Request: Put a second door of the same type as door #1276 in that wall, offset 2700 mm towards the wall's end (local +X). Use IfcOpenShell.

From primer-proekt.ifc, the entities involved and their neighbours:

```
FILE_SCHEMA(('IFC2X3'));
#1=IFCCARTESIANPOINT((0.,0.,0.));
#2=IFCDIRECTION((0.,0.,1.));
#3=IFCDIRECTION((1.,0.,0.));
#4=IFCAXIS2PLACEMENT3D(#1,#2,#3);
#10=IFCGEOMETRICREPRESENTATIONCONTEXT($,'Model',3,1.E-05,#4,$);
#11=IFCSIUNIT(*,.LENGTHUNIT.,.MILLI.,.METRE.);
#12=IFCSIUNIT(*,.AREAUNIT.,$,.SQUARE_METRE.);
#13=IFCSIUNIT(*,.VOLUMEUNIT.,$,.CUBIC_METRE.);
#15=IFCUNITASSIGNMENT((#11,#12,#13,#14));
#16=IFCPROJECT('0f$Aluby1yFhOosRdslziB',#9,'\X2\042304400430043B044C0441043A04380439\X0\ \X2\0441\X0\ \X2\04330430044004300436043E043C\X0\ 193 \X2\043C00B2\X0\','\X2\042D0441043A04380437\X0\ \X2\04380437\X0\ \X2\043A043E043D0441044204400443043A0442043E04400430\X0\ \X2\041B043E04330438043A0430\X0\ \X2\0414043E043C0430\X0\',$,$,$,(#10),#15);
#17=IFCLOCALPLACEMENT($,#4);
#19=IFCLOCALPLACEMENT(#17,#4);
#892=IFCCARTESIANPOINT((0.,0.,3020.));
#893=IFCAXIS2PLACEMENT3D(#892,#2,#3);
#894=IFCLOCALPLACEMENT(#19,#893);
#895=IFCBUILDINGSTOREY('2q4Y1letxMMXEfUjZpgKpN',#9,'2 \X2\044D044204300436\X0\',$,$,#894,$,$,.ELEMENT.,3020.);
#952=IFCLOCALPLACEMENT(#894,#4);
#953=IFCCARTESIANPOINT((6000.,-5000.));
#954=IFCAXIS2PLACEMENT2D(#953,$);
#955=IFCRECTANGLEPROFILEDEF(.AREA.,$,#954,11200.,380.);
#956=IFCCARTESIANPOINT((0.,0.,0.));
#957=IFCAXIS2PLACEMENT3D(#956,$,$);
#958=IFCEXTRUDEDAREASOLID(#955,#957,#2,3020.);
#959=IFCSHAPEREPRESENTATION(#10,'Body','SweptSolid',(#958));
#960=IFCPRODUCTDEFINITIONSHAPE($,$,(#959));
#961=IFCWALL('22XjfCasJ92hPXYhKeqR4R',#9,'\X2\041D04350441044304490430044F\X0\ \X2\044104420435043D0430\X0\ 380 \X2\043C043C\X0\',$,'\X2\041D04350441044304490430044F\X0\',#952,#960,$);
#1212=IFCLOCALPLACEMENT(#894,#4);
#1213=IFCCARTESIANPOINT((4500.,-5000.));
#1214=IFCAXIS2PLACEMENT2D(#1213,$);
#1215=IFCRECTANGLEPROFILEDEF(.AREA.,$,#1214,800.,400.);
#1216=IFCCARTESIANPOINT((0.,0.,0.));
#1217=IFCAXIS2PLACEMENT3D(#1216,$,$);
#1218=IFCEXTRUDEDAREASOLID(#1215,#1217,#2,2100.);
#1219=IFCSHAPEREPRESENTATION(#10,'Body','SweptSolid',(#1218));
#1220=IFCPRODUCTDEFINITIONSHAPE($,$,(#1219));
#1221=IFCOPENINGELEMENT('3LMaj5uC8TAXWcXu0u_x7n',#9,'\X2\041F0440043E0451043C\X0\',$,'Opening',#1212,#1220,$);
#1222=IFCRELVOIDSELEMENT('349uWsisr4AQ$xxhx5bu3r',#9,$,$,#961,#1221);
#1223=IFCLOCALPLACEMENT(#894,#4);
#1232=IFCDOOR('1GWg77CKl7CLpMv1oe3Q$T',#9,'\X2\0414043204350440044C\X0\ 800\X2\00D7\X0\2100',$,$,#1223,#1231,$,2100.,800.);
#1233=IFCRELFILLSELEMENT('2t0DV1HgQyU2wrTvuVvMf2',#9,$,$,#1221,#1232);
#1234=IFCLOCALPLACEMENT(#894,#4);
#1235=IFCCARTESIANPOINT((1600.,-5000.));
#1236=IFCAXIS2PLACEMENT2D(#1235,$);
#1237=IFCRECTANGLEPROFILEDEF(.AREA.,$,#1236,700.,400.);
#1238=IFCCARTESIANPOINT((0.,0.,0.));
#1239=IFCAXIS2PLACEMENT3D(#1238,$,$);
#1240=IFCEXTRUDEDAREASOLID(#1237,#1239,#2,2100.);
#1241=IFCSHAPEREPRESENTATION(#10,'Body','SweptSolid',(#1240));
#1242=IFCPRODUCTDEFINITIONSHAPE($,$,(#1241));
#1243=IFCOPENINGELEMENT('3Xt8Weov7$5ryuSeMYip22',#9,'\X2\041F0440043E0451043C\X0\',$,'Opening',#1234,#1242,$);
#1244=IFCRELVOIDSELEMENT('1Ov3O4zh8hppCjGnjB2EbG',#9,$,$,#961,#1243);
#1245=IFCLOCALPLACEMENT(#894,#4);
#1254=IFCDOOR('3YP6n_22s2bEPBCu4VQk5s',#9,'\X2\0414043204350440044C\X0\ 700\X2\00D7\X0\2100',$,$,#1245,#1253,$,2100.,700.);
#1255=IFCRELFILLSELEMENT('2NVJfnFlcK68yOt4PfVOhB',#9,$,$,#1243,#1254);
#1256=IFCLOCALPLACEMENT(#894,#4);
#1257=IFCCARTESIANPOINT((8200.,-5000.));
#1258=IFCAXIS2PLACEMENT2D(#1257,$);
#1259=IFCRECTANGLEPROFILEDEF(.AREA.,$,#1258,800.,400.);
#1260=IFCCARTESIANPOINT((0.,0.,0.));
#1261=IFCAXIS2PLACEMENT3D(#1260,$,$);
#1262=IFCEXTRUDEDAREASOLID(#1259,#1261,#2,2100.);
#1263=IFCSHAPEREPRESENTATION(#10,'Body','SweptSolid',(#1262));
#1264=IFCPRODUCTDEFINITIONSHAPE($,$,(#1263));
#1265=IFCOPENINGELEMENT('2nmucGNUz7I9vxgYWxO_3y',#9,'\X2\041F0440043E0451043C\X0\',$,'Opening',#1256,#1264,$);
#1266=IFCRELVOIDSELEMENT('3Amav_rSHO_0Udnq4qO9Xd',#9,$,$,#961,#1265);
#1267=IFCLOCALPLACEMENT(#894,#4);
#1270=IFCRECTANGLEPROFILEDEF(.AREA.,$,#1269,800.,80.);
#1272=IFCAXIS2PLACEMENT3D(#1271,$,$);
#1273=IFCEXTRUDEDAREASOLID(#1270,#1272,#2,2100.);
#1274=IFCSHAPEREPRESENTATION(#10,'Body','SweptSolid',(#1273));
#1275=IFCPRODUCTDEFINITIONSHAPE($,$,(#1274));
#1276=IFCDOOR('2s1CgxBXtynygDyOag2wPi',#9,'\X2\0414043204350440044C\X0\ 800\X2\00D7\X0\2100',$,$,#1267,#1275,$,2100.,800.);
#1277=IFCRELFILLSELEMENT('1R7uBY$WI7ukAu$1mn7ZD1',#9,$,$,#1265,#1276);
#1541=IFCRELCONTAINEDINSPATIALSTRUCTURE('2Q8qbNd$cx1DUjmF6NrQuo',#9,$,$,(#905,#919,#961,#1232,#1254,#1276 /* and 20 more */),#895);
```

```python
import ifcopenshell
import ifcopenshell.api.feature
import ifcopenshell.api.geometry
import ifcopenshell.api.root
import ifcopenshell.geom
import ifcopenshell.util.element
import ifcopenshell.util.placement
import ifcopenshell.util.shape

model = ifcopenshell.open("primer-proekt.ifc")
settings = ifcopenshell.geom.settings()


def volume(element):
    """Net volume in cubic metres, openings subtracted."""
    shape = ifcopenshell.geom.create_shape(settings, element)
    return ifcopenshell.util.shape.get_volume(shape.geometry)


door = model.by_guid("2s1CgxBXtynygDyOag2wPi")
opening = door.FillsVoids[0].RelatingOpeningElement
wall = opening.VoidsElements[0].RelatingBuildingElement
before = volume(wall)
shift = ifcopenshell.util.placement.get_local_placement(wall.ObjectPlacement)[:3, 0] * 2700.0

# copy_class copies the void relationship, type, container and properties, but no geometry.
new_opening = ifcopenshell.api.root.copy_class(model, product=opening)
new_opening.Representation = ifcopenshell.util.element.copy_deep(
    model, opening.Representation, exclude=["IfcGeometricRepresentationContext", "IfcRepresentationMap"]
)
new_door = ifcopenshell.api.root.copy_class(model, product=door)
new_door.Representation = ifcopenshell.util.element.copy_deep(
    model, door.Representation, exclude=["IfcGeometricRepresentationContext", "IfcRepresentationMap"]
)
fills = ifcopenshell.api.feature.add_filling(model, opening=new_opening, element=new_door)
fills.OwnerHistory = new_door.OwnerHistory  # required in IFC2X3

for old, new in ((opening, new_opening), (door, new_door)):
    matrix = ifcopenshell.util.placement.get_local_placement(old.ObjectPlacement)
    matrix[:3, 3] += shift
    ifcopenshell.api.geometry.edit_object_placement(model, product=new, matrix=matrix, is_si=False)

after = volume(wall)

print(f"wall volume {before:.3f} -> {after:.3f} m3")

model.write("primer-proekt_v2.ifc")
```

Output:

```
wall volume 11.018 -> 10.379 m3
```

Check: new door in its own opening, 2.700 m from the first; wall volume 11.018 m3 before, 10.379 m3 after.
